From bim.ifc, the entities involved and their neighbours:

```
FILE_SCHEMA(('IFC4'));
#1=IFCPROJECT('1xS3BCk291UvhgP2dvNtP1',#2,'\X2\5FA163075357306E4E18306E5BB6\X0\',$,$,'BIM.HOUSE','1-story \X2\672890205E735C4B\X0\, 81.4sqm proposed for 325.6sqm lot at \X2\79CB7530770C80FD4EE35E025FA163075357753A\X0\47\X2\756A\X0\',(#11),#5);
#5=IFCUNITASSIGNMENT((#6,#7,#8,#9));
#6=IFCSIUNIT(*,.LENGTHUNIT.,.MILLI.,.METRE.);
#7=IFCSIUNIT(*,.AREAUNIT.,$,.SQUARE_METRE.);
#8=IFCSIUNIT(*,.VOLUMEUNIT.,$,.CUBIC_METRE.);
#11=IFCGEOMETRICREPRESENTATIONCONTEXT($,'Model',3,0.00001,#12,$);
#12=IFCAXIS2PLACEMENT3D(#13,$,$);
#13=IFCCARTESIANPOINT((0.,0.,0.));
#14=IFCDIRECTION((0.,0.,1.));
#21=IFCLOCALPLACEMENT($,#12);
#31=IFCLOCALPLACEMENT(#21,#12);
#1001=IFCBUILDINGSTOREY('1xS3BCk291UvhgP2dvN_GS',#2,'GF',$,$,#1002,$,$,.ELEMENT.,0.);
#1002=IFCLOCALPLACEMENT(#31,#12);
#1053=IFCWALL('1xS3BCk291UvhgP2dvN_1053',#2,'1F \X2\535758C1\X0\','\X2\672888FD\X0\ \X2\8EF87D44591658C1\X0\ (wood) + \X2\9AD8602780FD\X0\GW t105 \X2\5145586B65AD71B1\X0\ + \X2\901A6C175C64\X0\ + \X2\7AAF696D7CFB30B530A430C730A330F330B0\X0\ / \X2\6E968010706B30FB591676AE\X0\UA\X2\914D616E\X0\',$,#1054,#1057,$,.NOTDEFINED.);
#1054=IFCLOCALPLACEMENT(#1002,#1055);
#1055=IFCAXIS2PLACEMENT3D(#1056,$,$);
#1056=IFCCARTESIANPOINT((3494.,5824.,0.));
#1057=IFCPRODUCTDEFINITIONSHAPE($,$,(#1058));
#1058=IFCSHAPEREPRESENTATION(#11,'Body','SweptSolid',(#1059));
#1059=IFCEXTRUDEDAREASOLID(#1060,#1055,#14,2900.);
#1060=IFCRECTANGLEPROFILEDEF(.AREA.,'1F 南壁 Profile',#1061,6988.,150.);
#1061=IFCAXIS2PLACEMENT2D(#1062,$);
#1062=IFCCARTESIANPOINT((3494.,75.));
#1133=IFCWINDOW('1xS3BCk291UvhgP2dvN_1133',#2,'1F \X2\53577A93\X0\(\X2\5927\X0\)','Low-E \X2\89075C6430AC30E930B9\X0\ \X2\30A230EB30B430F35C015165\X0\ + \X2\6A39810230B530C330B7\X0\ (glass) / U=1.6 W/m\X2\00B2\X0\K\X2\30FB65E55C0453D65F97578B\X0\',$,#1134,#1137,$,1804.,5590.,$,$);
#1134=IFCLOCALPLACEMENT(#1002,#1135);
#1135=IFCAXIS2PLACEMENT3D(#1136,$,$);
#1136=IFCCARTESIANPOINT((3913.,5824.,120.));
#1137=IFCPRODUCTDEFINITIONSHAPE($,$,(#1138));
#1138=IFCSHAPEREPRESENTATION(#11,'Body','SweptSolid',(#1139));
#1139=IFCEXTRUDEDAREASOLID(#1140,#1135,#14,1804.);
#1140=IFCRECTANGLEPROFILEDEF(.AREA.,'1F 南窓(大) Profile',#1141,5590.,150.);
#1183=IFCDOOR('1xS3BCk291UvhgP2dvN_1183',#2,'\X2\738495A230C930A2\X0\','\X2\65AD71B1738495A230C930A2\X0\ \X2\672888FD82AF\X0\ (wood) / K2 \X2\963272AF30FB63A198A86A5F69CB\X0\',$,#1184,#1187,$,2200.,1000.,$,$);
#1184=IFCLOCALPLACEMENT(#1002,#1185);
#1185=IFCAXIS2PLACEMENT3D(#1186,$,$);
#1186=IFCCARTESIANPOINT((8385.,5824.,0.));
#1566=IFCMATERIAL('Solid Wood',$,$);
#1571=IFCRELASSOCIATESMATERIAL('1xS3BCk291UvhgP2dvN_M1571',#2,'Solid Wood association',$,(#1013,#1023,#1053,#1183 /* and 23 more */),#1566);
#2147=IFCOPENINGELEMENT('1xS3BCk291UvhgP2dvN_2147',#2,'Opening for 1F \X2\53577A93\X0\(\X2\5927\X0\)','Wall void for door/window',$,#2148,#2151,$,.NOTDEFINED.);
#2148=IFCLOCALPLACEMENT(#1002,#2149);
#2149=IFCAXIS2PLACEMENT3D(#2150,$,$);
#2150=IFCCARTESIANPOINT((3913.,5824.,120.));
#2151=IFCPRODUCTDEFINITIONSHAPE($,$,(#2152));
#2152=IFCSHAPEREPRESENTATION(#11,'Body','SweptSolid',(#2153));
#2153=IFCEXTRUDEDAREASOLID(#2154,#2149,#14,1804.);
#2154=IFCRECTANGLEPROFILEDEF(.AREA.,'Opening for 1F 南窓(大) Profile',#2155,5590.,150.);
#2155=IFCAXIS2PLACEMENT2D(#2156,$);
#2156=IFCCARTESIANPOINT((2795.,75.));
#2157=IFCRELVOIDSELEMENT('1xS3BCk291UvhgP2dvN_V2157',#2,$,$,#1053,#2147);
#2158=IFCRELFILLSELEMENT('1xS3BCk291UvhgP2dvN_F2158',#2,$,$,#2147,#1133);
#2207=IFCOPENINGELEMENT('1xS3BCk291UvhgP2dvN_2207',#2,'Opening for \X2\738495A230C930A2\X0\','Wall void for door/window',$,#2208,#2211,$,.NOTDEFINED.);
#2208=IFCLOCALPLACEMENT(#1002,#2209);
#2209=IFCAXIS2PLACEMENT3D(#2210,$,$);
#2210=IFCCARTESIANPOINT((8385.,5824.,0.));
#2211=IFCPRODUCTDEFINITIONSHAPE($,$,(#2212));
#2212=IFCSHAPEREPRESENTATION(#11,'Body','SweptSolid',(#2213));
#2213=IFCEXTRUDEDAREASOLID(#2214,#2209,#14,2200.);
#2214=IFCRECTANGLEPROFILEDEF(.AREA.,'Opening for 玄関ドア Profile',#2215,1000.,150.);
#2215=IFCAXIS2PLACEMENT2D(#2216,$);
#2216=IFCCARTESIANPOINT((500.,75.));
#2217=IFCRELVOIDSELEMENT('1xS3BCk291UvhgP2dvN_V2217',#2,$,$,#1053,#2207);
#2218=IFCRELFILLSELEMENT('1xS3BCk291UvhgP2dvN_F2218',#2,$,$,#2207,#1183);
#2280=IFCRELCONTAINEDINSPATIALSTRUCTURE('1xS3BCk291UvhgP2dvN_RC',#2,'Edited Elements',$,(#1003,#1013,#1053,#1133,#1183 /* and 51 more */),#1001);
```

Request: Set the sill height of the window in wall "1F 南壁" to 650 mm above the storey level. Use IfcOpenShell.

```python
import numpy as np
import ifcopenshell
import ifcopenshell.api.geometry
import ifcopenshell.geom
import ifcopenshell.util.element
import ifcopenshell.util.placement
import ifcopenshell.util.shape
import ifcopenshell.util.unit

model = ifcopenshell.open("bim.ifc")
unit_scale = ifcopenshell.util.unit.calculate_unit_scale(model)

window = model.by_id(1133)
opening = window.FillsVoids[0].RelatingOpeningElement
storey = ifcopenshell.util.element.get_container(window, ifc_class="IfcBuildingStorey")
level = ifcopenshell.util.placement.get_local_placement(storey.ObjectPlacement)[2, 3]

# The opening's origin need not be at the sill, so measure its lowest point.
shape = ifcopenshell.geom.create_shape(ifcopenshell.geom.settings(), opening)
bottom = ifcopenshell.util.shape.get_shape_bottom_elevation(shape, shape.geometry) / unit_scale
dz = level + 0.65 / unit_scale - bottom

shift = np.array([0.0, 0.0, dz])
# The window is not placed relative to its opening, so move both.
for product in (opening, window):
    matrix = ifcopenshell.util.placement.get_local_placement(product.ObjectPlacement)
    matrix[:3, 3] += shift
    ifcopenshell.api.geometry.edit_object_placement(model, product=product, matrix=matrix, is_si=False)

print(f"moved by {dz * unit_scale:+.3f} m")

model.write("bim-out.ifc")
```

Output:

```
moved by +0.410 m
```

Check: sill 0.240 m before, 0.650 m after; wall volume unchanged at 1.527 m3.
